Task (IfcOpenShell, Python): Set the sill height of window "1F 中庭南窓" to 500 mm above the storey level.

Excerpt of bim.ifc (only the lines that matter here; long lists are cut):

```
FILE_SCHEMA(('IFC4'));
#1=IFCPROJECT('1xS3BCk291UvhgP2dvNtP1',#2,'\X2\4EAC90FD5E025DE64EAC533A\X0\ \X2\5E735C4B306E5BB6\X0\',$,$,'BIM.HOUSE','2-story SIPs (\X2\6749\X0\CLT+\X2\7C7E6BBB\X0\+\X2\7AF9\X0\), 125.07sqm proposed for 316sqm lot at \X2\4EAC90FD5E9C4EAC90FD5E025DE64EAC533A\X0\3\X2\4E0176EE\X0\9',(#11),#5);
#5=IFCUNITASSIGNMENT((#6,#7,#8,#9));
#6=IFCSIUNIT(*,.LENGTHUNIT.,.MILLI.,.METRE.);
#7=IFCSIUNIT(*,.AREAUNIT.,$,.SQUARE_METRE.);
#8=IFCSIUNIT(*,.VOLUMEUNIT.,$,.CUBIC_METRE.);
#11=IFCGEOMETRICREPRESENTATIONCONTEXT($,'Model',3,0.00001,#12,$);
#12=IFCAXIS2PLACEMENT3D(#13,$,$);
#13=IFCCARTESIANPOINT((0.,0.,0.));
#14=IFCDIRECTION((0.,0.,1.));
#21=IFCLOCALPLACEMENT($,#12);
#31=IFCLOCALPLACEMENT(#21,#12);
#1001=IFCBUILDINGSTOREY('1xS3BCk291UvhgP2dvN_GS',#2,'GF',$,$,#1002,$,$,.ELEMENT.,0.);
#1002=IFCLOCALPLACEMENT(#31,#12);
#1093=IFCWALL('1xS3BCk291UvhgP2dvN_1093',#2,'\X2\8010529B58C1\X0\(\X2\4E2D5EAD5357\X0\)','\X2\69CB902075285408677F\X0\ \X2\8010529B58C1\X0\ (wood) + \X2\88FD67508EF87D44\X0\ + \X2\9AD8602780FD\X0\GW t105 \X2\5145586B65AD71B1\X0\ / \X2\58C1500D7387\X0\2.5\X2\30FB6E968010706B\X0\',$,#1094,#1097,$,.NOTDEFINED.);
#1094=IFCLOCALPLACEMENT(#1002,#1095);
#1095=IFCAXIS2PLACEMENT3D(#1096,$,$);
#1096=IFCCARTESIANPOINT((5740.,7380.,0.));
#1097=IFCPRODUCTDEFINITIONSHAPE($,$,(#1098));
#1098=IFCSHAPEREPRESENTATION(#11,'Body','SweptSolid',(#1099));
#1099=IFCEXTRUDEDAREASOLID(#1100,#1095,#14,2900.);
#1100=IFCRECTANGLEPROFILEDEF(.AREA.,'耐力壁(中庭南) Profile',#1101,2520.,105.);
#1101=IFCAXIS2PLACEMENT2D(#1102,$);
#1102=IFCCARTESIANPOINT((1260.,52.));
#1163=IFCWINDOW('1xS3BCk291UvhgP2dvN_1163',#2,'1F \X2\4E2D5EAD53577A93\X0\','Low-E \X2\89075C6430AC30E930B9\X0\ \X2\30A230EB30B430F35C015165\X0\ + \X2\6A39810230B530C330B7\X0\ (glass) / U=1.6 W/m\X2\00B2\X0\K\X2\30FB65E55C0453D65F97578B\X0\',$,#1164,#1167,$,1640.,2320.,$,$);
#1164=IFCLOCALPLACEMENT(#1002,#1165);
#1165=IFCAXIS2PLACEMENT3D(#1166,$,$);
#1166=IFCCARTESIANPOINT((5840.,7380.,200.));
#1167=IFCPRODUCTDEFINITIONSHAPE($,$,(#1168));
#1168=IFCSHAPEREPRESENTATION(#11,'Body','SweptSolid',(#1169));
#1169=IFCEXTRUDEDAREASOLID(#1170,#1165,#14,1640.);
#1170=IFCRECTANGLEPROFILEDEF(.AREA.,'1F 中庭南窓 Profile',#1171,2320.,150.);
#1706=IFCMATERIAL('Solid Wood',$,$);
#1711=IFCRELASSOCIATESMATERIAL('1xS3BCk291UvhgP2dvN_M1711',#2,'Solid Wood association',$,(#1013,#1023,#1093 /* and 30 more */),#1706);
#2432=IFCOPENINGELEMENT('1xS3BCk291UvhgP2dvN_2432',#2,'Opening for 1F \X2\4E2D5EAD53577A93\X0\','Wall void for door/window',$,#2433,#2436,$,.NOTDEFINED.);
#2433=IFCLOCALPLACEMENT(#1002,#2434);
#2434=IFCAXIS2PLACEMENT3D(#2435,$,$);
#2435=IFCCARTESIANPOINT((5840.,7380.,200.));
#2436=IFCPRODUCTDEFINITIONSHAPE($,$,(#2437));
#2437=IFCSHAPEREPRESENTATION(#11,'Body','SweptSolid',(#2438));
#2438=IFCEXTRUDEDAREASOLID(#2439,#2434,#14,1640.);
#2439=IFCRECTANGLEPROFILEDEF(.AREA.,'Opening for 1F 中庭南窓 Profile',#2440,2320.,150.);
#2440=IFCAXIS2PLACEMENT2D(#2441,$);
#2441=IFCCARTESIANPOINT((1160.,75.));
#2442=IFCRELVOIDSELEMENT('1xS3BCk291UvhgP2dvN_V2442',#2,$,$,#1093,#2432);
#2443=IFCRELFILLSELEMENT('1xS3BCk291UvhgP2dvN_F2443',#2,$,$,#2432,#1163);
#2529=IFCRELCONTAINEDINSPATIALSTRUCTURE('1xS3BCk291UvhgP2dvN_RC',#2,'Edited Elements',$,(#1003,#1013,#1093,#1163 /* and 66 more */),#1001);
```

```python
import numpy as np
import ifcopenshell
import ifcopenshell.api.geometry
import ifcopenshell.geom
import ifcopenshell.util.element
import ifcopenshell.util.placement
import ifcopenshell.util.shape
import ifcopenshell.util.unit

model = ifcopenshell.open("bim.ifc")
unit_scale = ifcopenshell.util.unit.calculate_unit_scale(model)

window = model.by_id(1163)
opening = window.FillsVoids[0].RelatingOpeningElement
storey = ifcopenshell.util.element.get_container(window, ifc_class="IfcBuildingStorey")
level = ifcopenshell.util.placement.get_local_placement(storey.ObjectPlacement)[2, 3]

# The opening's origin need not be at the sill, so measure its lowest point.
shape = ifcopenshell.geom.create_shape(ifcopenshell.geom.settings(), opening)
bottom = ifcopenshell.util.shape.get_shape_bottom_elevation(shape, shape.geometry) / unit_scale
dz = level + 0.5 / unit_scale - bottom

shift = np.array([0.0, 0.0, dz])
# The window is not placed relative to its opening, so move both.
for product in (opening, window):
    matrix = ifcopenshell.util.placement.get_local_placement(product.ObjectPlacement)
    matrix[:3, 3] += shift
    ifcopenshell.api.geometry.edit_object_placement(model, product=product, matrix=matrix, is_si=False)

print(f"moved by {dz * unit_scale:+.3f} m")

model.write("bim_v2.ifc")
```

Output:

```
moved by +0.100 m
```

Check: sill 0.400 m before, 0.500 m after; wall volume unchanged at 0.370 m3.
